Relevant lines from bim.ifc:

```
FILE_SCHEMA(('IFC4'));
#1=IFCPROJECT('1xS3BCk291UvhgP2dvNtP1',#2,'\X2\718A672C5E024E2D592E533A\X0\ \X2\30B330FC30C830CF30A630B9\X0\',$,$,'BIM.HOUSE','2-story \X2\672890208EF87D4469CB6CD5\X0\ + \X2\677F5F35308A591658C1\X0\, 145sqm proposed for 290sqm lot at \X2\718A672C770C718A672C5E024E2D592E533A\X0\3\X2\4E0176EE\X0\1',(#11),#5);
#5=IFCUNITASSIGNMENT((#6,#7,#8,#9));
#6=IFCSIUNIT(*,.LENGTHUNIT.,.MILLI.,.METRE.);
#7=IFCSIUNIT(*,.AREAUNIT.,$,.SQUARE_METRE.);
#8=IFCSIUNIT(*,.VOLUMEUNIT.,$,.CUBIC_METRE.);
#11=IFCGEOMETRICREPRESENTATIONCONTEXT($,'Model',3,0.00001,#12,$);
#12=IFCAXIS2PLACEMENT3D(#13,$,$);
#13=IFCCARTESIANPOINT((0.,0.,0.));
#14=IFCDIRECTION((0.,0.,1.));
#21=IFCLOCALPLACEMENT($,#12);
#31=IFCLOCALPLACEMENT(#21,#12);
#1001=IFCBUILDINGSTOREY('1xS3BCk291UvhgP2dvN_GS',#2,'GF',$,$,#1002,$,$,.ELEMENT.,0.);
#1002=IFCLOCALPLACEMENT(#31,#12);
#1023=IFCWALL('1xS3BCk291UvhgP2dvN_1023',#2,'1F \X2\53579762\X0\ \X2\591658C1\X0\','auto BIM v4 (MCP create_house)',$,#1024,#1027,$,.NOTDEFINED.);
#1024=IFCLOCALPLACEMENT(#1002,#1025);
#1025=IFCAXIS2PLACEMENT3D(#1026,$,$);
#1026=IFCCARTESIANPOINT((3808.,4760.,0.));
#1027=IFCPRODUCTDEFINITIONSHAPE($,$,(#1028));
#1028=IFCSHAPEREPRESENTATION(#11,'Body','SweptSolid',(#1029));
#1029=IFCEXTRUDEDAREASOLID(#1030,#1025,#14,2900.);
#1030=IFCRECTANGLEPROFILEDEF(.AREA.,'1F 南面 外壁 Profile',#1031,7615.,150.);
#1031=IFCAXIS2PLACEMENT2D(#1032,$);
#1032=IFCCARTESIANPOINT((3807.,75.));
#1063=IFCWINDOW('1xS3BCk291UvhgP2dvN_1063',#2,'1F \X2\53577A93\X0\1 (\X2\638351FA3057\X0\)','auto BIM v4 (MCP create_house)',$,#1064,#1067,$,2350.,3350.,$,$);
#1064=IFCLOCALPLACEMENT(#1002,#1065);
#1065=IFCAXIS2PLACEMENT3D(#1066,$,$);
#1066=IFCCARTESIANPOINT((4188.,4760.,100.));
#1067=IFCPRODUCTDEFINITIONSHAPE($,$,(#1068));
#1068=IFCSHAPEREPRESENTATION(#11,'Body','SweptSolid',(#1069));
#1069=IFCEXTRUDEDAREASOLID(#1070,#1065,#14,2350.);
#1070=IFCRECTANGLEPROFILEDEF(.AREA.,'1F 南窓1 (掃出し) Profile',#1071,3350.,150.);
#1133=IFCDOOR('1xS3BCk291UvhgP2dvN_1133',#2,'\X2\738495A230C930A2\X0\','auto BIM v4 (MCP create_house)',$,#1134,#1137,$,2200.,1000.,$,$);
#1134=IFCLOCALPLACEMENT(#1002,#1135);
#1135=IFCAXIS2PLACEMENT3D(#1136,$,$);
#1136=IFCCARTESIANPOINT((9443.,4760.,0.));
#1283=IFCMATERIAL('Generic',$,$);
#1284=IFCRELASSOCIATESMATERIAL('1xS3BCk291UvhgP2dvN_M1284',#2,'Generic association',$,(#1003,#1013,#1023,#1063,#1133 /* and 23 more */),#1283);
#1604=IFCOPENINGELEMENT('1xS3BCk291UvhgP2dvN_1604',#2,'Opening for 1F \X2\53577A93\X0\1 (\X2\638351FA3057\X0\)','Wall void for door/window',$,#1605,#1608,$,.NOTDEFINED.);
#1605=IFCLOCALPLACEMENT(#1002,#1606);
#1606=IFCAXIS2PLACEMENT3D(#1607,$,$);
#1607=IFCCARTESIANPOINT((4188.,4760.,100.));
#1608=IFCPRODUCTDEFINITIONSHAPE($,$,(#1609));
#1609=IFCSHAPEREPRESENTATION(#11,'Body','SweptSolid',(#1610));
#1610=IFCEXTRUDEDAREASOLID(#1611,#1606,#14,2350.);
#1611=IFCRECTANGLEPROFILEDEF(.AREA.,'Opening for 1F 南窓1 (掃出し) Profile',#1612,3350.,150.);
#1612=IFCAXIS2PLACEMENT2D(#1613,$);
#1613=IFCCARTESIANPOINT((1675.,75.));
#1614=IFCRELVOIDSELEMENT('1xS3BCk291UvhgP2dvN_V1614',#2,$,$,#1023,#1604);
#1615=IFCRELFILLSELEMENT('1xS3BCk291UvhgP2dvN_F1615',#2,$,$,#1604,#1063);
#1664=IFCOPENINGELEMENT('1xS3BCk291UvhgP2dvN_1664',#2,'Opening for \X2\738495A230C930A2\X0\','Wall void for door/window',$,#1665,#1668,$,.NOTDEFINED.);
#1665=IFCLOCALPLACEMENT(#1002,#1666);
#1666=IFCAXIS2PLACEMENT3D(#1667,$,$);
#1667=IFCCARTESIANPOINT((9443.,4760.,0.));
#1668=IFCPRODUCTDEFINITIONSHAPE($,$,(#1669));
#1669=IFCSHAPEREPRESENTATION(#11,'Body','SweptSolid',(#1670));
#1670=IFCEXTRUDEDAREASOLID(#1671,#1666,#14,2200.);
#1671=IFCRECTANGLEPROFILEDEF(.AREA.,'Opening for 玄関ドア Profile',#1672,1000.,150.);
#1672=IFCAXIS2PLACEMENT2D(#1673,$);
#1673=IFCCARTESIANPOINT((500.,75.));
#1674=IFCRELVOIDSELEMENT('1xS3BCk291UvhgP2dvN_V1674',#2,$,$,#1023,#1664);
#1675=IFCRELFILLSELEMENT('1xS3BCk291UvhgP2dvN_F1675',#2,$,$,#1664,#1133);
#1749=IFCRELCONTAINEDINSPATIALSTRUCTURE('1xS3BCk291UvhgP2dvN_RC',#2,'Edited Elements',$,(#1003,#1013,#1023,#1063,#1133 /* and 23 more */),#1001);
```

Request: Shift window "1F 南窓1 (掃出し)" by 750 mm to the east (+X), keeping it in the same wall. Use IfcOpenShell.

```python
import ifcopenshell
import ifcopenshell.api.geometry
import ifcopenshell.util.placement

model = ifcopenshell.open("bim.ifc")

window = model.by_guid("1xS3BCk291UvhgP2dvN_1063")
opening = window.FillsVoids[0].RelatingOpeningElement
wall = opening.VoidsElements[0].RelatingBuildingElement

wall_matrix = ifcopenshell.util.placement.get_local_placement(wall.ObjectPlacement)
shift = wall_matrix[:3, 0] * 750.0
before = ifcopenshell.util.placement.get_local_placement(window.ObjectPlacement)[:3, 3].copy()

# The window is not placed relative to its opening, so move both.
for product in (opening, window):
    matrix = ifcopenshell.util.placement.get_local_placement(product.ObjectPlacement)
    matrix[:3, 3] += shift
    ifcopenshell.api.geometry.edit_object_placement(model, product=product, matrix=matrix, is_si=False)

after = ifcopenshell.util.placement.get_local_placement(window.ObjectPlacement)[:3, 3]
print("window moved by", (after - before).round(3) + 0.0)

model.write("bim_edited.ifc")
```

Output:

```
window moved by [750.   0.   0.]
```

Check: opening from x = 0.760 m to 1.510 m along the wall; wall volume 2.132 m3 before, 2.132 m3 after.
